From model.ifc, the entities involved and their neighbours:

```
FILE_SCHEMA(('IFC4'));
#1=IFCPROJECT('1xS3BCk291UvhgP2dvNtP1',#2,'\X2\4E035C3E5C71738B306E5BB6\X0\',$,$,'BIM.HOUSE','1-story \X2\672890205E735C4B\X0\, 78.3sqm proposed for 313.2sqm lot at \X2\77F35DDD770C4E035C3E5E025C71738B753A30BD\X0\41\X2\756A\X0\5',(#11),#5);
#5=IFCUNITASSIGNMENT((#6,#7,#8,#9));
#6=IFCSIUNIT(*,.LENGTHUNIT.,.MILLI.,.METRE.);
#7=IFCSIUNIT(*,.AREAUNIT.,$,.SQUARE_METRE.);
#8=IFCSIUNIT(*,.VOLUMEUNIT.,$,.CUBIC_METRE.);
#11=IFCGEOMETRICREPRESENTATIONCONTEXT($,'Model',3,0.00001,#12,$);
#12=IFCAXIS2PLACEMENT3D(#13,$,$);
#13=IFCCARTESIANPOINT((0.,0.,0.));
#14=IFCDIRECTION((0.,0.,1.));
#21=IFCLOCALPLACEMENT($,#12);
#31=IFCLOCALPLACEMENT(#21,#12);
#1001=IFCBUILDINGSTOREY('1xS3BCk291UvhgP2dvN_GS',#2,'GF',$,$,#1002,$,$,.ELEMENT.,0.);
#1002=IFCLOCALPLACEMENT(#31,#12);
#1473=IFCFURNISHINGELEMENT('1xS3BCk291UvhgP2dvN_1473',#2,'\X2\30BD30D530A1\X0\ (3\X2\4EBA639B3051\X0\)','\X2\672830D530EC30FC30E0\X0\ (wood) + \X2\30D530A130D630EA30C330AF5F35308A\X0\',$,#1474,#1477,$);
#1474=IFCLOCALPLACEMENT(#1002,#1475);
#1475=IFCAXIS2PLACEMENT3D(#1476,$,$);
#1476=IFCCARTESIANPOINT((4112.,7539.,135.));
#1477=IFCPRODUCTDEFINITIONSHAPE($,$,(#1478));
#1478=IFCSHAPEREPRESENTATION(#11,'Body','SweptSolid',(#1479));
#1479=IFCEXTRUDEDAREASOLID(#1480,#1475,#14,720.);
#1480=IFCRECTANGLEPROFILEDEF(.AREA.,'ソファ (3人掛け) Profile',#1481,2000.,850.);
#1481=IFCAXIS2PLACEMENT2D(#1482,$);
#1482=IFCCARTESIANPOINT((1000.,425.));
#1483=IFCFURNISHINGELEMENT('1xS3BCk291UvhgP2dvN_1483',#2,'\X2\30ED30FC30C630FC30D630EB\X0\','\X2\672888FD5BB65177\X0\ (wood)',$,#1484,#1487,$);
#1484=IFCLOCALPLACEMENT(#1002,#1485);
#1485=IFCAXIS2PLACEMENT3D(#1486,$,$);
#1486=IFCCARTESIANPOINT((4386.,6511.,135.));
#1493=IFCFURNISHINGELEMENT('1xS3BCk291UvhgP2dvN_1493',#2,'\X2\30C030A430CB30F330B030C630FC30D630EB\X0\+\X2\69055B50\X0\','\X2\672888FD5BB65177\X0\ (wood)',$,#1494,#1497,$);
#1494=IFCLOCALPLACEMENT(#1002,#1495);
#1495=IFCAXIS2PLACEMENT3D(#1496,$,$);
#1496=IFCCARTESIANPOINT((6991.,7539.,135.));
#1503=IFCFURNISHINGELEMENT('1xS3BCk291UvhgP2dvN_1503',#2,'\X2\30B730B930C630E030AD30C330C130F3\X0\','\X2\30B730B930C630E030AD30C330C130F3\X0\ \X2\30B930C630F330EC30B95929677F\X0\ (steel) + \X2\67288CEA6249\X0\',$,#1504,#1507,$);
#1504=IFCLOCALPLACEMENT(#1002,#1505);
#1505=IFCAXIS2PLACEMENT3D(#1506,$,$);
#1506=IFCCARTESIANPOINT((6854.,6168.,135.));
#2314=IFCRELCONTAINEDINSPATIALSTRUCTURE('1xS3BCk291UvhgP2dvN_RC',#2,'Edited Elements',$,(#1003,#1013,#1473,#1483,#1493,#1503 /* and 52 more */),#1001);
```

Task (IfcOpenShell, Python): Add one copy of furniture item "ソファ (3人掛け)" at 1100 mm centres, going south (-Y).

```python
import numpy as np
import ifcopenshell
import ifcopenshell.api.geometry
import ifcopenshell.api.root
import ifcopenshell.util.element
import ifcopenshell.util.placement
import ifcopenshell.util.unit

model = ifcopenshell.open("model.ifc")
unit_scale = ifcopenshell.util.unit.calculate_unit_scale(model)


def reuse_history(source, copy):
    """copy_class also copies each property set's owner history, people and application; keep the originals."""
    for rel in copy.IsDefinedBy:
        if rel.is_a("IfcRelDefinesByProperties") and (history := rel.RelatingPropertyDefinition.OwnerHistory):
            rel.RelatingPropertyDefinition.OwnerHistory = source.OwnerHistory
            ifcopenshell.util.element.remove_deep2(model, history)


source = model.by_guid("1xS3BCk291UvhgP2dvN_1473")
base = ifcopenshell.util.placement.get_local_placement(source.ObjectPlacement)
step = np.array([0.0, -1.0, 0.0]) * 1.1 / unit_scale

for i in range(1, 2):
    copy = ifcopenshell.api.root.copy_class(model, product=source)
    copy.Representation = ifcopenshell.util.element.copy_deep(
        model, source.Representation, exclude=["IfcGeometricRepresentationContext", "IfcRepresentationMap"]
    )
    reuse_history(source, copy)
    matrix = base.copy()
    matrix[:3, 3] += i * step
    print("added at", matrix[:3, 3].round(3) + 0.0)
    ifcopenshell.api.geometry.edit_object_placement(model, product=copy, matrix=matrix, is_si=False)

model.write("model_edited.ifc")
```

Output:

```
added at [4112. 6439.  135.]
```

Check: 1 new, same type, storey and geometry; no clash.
